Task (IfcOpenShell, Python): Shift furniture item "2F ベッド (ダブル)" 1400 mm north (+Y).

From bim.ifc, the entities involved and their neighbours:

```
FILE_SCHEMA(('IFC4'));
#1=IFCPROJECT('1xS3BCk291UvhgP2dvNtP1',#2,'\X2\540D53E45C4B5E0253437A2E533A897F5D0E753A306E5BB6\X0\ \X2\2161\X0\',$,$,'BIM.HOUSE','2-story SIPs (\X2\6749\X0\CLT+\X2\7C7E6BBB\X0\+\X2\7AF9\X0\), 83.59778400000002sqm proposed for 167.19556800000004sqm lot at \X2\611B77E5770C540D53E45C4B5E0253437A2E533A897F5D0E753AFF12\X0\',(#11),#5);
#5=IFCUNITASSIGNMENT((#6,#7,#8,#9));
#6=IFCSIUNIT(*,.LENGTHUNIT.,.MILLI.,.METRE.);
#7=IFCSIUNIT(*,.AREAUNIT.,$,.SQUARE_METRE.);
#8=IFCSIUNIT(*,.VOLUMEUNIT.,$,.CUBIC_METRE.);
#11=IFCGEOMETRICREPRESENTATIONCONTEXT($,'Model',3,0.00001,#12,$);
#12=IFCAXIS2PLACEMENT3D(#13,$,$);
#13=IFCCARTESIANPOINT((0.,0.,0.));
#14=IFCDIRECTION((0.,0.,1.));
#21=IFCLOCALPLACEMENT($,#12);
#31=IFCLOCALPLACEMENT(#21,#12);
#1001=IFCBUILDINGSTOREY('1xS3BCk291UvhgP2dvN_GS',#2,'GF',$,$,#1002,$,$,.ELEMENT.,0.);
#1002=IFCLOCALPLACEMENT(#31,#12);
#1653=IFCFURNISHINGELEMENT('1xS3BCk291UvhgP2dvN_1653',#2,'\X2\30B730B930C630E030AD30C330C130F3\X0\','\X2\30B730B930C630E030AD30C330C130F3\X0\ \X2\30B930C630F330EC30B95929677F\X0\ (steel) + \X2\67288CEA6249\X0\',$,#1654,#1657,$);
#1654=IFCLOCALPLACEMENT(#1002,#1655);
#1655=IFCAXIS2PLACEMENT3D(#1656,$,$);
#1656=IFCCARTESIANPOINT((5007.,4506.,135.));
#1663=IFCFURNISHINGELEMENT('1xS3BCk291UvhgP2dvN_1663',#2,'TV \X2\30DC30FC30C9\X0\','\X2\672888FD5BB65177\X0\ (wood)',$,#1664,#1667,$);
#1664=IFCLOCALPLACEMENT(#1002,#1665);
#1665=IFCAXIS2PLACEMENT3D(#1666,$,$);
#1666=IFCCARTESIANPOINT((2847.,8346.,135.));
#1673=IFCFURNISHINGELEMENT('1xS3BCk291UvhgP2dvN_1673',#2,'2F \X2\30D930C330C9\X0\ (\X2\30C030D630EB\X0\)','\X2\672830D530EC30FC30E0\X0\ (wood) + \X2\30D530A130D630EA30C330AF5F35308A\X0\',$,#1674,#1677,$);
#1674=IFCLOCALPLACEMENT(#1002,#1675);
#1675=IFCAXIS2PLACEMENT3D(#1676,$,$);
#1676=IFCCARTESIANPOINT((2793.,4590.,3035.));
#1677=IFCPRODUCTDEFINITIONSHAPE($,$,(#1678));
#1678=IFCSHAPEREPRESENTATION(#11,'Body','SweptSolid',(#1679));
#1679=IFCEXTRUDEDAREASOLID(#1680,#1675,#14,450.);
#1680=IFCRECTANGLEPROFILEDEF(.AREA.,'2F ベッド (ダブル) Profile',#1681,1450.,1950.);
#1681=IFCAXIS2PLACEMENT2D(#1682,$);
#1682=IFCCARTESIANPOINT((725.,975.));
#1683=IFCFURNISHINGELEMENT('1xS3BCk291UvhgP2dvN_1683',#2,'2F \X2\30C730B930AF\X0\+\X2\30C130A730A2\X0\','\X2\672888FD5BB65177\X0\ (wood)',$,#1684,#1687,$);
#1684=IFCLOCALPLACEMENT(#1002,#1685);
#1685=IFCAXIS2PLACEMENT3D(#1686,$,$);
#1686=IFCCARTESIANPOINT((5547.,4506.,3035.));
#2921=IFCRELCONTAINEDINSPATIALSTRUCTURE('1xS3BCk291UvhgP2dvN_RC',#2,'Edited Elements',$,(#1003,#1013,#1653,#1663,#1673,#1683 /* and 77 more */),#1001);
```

```python
import ifcopenshell
import ifcopenshell.api.geometry
import ifcopenshell.util.placement

model = ifcopenshell.open("bim.ifc")

item = model.by_guid("1xS3BCk291UvhgP2dvN_1673")
matrix = ifcopenshell.util.placement.get_local_placement(item.ObjectPlacement)
matrix[1, 3] += 1400.0
ifcopenshell.api.geometry.edit_object_placement(model, product=item, matrix=matrix, is_si=False)

print(ifcopenshell.util.placement.get_local_placement(item.ObjectPlacement).round(3) + 0.0)

model.write("bim_v2.ifc")
```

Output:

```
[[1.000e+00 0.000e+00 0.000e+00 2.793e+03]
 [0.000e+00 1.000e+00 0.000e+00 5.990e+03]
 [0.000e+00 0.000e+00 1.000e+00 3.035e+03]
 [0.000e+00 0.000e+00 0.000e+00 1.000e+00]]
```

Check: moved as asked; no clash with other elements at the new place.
